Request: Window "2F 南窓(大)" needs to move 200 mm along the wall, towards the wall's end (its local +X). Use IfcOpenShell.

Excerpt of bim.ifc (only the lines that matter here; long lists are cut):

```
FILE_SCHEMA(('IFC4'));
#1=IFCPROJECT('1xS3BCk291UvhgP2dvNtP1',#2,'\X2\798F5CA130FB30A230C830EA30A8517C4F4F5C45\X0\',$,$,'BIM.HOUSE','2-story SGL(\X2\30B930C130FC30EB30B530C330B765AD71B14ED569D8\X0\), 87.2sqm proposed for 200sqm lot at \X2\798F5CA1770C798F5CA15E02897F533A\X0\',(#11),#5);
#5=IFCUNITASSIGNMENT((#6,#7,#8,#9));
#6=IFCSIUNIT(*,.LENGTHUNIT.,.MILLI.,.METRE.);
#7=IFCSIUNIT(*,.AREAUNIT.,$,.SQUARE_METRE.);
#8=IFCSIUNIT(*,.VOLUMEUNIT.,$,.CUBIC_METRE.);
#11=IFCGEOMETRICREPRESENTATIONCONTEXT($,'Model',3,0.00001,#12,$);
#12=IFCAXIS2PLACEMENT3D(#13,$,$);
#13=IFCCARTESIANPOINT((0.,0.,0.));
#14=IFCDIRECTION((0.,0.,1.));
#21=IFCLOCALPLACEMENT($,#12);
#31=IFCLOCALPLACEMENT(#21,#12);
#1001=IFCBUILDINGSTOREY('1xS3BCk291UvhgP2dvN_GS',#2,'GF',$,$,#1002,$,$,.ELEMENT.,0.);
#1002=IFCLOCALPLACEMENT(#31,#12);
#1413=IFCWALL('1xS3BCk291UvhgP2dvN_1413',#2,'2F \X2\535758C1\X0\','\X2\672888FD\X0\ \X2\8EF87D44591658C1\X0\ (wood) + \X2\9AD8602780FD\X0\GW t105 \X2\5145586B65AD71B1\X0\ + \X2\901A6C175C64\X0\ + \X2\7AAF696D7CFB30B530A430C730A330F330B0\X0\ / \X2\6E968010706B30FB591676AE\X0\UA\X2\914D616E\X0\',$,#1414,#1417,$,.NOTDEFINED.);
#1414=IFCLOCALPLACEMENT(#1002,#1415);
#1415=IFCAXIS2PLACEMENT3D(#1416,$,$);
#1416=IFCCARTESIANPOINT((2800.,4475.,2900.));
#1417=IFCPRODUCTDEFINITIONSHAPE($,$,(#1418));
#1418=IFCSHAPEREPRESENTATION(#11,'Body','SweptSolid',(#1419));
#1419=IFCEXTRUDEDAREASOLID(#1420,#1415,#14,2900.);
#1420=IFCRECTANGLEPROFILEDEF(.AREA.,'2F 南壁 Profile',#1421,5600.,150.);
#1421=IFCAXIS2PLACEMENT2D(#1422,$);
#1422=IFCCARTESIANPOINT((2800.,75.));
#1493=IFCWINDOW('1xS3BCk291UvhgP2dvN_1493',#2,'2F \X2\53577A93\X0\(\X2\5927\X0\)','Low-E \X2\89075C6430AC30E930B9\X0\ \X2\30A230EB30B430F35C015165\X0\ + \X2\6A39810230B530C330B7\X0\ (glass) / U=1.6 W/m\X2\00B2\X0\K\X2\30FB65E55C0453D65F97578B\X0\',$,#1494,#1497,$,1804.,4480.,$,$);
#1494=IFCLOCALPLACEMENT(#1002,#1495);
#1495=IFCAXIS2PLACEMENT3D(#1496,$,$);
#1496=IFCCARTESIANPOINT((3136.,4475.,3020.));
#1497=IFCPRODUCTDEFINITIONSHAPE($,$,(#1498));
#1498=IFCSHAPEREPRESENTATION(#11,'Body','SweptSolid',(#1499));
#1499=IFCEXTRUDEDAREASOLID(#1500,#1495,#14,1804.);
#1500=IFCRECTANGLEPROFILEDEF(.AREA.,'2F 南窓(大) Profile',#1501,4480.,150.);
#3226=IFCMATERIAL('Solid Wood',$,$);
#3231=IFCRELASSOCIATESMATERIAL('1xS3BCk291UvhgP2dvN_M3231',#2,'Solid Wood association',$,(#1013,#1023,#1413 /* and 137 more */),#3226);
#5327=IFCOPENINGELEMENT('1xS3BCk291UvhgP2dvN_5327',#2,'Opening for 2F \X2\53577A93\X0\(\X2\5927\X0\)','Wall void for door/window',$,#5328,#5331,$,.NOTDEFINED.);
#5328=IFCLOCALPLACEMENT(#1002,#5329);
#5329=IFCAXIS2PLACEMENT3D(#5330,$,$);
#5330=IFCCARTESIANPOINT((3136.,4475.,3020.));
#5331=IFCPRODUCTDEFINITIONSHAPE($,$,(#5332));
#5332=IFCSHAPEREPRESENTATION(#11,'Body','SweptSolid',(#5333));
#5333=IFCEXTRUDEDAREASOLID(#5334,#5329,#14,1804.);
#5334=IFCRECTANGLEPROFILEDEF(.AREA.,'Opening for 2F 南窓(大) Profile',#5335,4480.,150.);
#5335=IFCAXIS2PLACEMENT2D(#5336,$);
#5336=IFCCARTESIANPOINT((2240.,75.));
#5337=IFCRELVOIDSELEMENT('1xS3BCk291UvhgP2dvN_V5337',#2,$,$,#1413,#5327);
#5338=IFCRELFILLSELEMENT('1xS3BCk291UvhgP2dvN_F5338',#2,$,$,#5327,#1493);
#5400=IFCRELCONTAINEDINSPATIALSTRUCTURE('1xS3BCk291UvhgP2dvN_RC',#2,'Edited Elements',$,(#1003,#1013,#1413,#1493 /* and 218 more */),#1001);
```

```python
import ifcopenshell
import ifcopenshell.api.geometry
import ifcopenshell.util.placement

model = ifcopenshell.open("bim.ifc")

window = model.by_id(1493)
opening = window.FillsVoids[0].RelatingOpeningElement
wall = opening.VoidsElements[0].RelatingBuildingElement

wall_matrix = ifcopenshell.util.placement.get_local_placement(wall.ObjectPlacement)
shift = wall_matrix[:3, 0] * 200.0
before = ifcopenshell.util.placement.get_local_placement(window.ObjectPlacement)[:3, 3].copy()

# The window is not placed relative to its opening, so move both.
for product in (opening, window):
    matrix = ifcopenshell.util.placement.get_local_placement(product.ObjectPlacement)
    matrix[:3, 3] += shift
    ifcopenshell.api.geometry.edit_object_placement(model, product=product, matrix=matrix, is_si=False)

after = ifcopenshell.util.placement.get_local_placement(window.ObjectPlacement)[:3, 3]
print("window moved by", (after - before).round(3) + 0.0)

model.write("bim_edited.ifc")
```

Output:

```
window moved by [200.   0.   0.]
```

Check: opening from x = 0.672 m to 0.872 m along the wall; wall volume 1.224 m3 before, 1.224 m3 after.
